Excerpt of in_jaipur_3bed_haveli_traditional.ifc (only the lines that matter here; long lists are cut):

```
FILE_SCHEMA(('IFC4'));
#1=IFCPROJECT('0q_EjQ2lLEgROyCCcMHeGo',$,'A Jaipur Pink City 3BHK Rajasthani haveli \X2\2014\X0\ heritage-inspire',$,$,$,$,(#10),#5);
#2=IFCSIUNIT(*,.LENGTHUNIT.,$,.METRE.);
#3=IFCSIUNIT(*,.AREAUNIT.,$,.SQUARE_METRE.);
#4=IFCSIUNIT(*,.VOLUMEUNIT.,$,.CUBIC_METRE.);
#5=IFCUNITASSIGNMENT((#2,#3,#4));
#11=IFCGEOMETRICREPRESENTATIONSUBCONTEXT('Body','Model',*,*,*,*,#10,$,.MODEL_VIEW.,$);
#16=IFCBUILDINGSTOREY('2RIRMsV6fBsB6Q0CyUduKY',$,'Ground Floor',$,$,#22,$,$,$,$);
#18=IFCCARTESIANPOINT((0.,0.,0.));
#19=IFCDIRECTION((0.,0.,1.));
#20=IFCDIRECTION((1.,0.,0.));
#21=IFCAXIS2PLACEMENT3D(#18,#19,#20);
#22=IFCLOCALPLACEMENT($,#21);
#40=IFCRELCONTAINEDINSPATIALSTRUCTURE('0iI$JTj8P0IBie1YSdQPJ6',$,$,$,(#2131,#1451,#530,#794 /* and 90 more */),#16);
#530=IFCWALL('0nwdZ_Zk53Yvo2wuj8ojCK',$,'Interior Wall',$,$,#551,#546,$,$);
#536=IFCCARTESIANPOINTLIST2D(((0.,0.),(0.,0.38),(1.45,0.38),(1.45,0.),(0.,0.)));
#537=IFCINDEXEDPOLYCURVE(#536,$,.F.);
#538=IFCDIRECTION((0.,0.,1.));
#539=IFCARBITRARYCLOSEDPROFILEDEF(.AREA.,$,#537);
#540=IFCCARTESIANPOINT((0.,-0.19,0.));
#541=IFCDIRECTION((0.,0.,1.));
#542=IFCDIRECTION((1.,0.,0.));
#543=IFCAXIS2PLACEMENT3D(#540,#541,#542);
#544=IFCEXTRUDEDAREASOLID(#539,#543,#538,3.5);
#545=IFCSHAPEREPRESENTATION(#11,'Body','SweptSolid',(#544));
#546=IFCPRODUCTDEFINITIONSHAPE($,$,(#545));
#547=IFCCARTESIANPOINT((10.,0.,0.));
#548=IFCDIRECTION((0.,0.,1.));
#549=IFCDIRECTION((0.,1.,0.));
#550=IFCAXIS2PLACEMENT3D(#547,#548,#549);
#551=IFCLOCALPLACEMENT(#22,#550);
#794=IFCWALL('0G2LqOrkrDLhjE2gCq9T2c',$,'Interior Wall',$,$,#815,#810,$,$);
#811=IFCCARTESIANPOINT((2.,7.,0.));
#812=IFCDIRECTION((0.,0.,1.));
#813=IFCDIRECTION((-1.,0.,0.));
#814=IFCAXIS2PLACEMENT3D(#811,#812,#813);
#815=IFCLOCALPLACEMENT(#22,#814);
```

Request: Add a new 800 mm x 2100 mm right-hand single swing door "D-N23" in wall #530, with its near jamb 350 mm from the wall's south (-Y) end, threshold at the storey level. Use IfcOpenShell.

```python
import numpy as np
import ifcopenshell
import ifcopenshell.api.feature
import ifcopenshell.api.geometry
import ifcopenshell.api.root
import ifcopenshell.api.spatial
import ifcopenshell.geom
import ifcopenshell.util.element
import ifcopenshell.util.placement
import ifcopenshell.util.representation
import ifcopenshell.util.shape
import ifcopenshell.util.unit

model = ifcopenshell.open("in_jaipur_3bed_haveli_traditional.ifc")
unit_scale = ifcopenshell.util.unit.calculate_unit_scale(model)
settings = ifcopenshell.geom.settings()


def volume(element):
    """Net volume in cubic metres, openings subtracted."""
    shape = ifcopenshell.geom.create_shape(settings, element)
    return ifcopenshell.util.shape.get_volume(shape.geometry)


wall = model.by_guid("0nwdZ_Zk53Yvo2wuj8ojCK")
storey = ifcopenshell.util.element.get_container(wall, ifc_class="IfcBuildingStorey")
context = ifcopenshell.util.representation.get_context(model, "Model", "Body", "MODEL_VIEW")
before = volume(wall)

width, height, from_end, sill = 0.8, 2.1, 0.35, 0.0  # metres

# The wall runs along its own X axis, and the end named is its -X end.
wall_shape = ifcopenshell.geom.create_shape(settings, wall)
x, y, z = ifcopenshell.util.shape.get_vertices(wall_shape.geometry).T
start = x.min() + from_end
face, thickness = float(y.min()), float(y.max() - y.min())
wall_matrix = ifcopenshell.util.placement.get_local_placement(wall.ObjectPlacement)
level = ifcopenshell.util.placement.get_local_placement(storey.ObjectPlacement)[2, 3]


def in_wall(x, y):
    """Placement at x, y metres in the wall's axes, at sill height."""
    matrix = wall_matrix.copy()
    matrix[:, 3] = wall_matrix @ np.array([x / unit_scale, y / unit_scale, 0.0, 1.0])
    matrix[2, 3] = level + sill / unit_scale
    return matrix


# Opening: a box that overshoots both wall faces by 50 mm.
opening = ifcopenshell.api.root.create_entity(model, ifc_class="IfcOpeningElement", predefined_type="OPENING")
box = ifcopenshell.api.geometry.add_wall_representation(
    model, context=context, length=width, height=height, thickness=thickness + 0.1
)
ifcopenshell.api.geometry.assign_representation(model, product=opening, representation=box)
ifcopenshell.api.geometry.edit_object_placement(model, product=opening, matrix=in_wall(start, face - 0.05), is_si=False)
ifcopenshell.api.feature.add_feature(model, feature=opening, element=wall)

door = ifcopenshell.api.root.create_entity(model, ifc_class="IfcDoor", name="D-N23", predefined_type="DOOR")
door.OverallWidth, door.OverallHeight = width / unit_scale, height / unit_scale
door.OperationType = "SINGLE_SWING_RIGHT"
body = ifcopenshell.api.geometry.add_door_representation(
    model,
    context=context,
    overall_width=door.OverallWidth,
    overall_height=door.OverallHeight,
    operation_type="SINGLE_SWING_RIGHT",
    lining_properties={"LiningDepth": thickness / unit_scale, "ThresholdDepth": thickness / unit_scale},
)
ifcopenshell.api.geometry.assign_representation(model, product=door, representation=body)
ifcopenshell.api.spatial.assign_container(model, products=[door], relating_structure=storey)
ifcopenshell.api.feature.add_filling(model, opening=opening, element=door)

# The lining spans the wall, so the door starts at the wall face.
ifcopenshell.api.geometry.edit_object_placement(model, product=door, matrix=in_wall(start, face), is_si=False)

after = volume(wall)

print(f"wall volume {before:.3f} -> {after:.3f} m3")

model.write("in_jaipur_3bed_haveli_traditional_edited.ifc")
```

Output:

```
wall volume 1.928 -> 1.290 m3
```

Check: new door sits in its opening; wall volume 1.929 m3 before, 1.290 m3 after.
